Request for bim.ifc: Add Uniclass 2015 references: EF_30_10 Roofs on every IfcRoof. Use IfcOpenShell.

First a look at what the model holds.

```python
import ifcopenshell

model = ifcopenshell.open("bim.ifc")
print(model.schema)
print("classifications:", [c.Name for c in model.by_type("IfcClassification")])
for ifc_class in ("IfcDoor", "IfcRoof", "IfcStair", "IfcWall", "IfcWindow"):
    print(ifc_class, len(model.by_type(ifc_class)))
```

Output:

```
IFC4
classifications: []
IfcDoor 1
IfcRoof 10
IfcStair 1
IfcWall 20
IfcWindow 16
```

```python
import ifcopenshell
import ifcopenshell.api.classification

model = ifcopenshell.open("bim.ifc")

system = ifcopenshell.api.classification.add_classification(model, classification="Uniclass 2015")

codes = {
    "IfcRoof": ("EF_30_10", "Roofs"),
}
for ifc_class, (code, name) in codes.items():
    products = model.by_type(ifc_class)
    ifcopenshell.api.classification.add_reference(
        model, products=products, classification=system, identification=code, name=name
    )
    print(code, len(products))

model.write("bim_v2.ifc")
```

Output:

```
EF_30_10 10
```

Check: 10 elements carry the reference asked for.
